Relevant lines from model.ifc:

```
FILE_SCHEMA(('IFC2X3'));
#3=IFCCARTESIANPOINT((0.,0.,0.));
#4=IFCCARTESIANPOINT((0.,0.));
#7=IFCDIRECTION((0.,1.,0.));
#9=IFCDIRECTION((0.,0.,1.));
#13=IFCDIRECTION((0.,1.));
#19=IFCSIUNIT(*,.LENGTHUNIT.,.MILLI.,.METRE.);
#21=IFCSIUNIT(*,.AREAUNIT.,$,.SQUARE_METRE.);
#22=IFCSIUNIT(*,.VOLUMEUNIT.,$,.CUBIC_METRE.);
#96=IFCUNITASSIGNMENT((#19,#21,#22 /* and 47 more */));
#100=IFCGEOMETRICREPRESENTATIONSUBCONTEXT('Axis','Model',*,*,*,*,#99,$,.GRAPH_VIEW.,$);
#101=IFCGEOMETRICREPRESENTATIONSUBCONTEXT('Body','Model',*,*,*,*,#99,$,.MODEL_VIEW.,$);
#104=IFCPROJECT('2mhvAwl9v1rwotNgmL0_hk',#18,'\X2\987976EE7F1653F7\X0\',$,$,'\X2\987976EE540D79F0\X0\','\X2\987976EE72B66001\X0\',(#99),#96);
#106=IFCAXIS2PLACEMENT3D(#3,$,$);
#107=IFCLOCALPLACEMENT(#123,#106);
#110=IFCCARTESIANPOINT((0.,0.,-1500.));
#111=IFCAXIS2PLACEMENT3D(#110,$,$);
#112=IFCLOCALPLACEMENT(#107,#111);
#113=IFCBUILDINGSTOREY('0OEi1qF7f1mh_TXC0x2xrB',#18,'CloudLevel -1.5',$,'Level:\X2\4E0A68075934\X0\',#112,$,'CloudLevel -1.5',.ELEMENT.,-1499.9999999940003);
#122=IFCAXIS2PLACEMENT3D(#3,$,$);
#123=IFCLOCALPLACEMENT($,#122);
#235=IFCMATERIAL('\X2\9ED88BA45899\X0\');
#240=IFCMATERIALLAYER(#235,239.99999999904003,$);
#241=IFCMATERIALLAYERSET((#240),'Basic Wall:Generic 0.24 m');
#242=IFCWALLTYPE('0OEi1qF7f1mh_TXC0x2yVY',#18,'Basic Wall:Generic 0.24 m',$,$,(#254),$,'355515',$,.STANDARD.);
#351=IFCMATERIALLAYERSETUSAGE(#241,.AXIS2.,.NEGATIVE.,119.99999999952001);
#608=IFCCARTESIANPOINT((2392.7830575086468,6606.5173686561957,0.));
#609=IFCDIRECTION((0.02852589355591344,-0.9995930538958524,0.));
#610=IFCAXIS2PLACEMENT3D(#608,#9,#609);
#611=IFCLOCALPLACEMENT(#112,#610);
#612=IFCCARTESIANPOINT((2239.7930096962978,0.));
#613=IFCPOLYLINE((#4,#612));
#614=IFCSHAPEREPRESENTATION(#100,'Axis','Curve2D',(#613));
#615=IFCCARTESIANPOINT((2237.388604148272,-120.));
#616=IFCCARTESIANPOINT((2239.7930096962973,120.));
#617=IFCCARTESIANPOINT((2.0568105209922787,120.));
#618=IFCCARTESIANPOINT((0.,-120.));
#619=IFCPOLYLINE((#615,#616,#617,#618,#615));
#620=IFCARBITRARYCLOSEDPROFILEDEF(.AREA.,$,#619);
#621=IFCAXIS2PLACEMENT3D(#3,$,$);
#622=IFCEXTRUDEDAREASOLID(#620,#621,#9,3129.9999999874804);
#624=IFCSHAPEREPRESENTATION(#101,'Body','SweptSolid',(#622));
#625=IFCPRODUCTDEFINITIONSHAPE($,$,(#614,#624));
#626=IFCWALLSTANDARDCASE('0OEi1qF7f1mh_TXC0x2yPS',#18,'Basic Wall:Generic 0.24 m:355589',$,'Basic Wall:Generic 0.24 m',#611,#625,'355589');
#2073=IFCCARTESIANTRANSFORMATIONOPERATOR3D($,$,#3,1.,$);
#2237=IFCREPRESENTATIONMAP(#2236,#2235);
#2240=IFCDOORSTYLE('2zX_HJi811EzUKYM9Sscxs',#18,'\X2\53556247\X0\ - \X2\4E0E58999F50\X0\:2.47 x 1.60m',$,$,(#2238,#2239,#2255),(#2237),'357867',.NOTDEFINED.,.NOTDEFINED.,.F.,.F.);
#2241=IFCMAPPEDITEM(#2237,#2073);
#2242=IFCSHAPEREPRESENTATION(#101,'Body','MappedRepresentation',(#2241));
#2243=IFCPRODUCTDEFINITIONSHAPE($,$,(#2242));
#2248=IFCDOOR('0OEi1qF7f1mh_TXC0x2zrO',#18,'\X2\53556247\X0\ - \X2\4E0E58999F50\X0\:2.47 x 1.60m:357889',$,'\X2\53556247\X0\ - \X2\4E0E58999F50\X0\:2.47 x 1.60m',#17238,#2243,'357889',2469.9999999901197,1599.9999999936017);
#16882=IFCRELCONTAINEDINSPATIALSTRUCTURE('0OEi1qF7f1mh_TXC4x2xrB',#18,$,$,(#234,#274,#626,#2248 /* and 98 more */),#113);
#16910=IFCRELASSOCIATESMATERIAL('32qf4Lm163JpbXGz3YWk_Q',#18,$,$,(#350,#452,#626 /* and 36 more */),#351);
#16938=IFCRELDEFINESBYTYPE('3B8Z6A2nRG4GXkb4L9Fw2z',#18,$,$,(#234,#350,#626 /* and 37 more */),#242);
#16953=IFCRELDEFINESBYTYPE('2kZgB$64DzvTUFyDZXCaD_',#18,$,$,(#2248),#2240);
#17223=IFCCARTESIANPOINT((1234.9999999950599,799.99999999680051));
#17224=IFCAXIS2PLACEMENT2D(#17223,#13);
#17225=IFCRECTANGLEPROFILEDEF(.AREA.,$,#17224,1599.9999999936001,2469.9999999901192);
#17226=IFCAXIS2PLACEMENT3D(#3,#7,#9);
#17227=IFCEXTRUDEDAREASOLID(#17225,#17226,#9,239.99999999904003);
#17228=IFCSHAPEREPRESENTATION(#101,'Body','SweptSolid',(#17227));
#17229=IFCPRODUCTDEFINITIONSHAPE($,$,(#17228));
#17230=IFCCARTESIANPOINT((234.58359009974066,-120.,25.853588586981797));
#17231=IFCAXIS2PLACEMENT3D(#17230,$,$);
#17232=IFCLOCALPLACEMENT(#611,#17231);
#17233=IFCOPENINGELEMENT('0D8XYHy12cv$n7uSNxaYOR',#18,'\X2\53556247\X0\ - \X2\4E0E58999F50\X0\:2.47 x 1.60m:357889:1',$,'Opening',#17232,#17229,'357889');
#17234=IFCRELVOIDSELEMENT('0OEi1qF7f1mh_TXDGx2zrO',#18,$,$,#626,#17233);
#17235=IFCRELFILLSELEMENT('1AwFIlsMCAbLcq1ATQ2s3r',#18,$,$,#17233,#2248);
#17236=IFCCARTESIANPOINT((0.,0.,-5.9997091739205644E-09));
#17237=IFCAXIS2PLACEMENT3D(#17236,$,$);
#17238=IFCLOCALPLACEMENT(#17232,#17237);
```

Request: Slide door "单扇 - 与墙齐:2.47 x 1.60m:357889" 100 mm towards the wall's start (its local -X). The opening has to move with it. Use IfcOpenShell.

```python
import ifcopenshell
import ifcopenshell.api.geometry
import ifcopenshell.util.placement
import ifcopenshell.util.unit

model = ifcopenshell.open("model.ifc")
unit_scale = ifcopenshell.util.unit.calculate_unit_scale(model)

door = model.by_guid("0OEi1qF7f1mh_TXC0x2zrO")
opening = door.FillsVoids[0].RelatingOpeningElement
wall = opening.VoidsElements[0].RelatingBuildingElement

wall_matrix = ifcopenshell.util.placement.get_local_placement(wall.ObjectPlacement)
shift = wall_matrix[:3, 0] * -0.1 / unit_scale
before = ifcopenshell.util.placement.get_local_placement(door.ObjectPlacement)[:3, 3].copy()

# The door is placed relative to its opening, so it follows when the opening moves.
matrix = ifcopenshell.util.placement.get_local_placement(opening.ObjectPlacement)
matrix[:3, 3] += shift
ifcopenshell.api.geometry.edit_object_placement(
    model, product=opening, matrix=matrix, is_si=False, should_transform_children=True
)

after = ifcopenshell.util.placement.get_local_placement(door.ObjectPlacement)[:3, 3]
print("door moved by", (after - before).round(3) + 0.0)

model.write("model-out.ifc")
```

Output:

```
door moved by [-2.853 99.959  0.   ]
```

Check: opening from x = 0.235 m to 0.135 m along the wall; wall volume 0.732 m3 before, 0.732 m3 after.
